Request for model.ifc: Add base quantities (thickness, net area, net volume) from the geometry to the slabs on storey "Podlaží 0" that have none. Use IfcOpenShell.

First a look at what the model holds.

```python
import ifcopenshell
import ifcopenshell.util.element
import ifcopenshell.util.unit

model = ifcopenshell.open("model.ifc")
print(model.schema)
for unit_type in ("LENGTHUNIT", "AREAUNIT", "VOLUMEUNIT"):
    print(unit_type, ifcopenshell.util.unit.calculate_unit_scale(model, unit_type))
storey = next(s for s in model.by_type("IfcBuildingStorey") if s.Name == "Podlaží 0")
slabs = [e for e in ifcopenshell.util.element.get_decomposition(storey) if e.is_a("IfcSlab")]
for e in sorted(slabs, key=lambda e: e.id()):
    print(e.id(), e.is_a(), e.Name, list(ifcopenshell.util.element.get_psets(e, qtos_only=True)), sep=" | ")
```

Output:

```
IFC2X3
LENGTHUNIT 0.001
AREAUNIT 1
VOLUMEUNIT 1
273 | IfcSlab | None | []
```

```python
import ifcopenshell
import ifcopenshell.api.pset
import ifcopenshell.geom
import ifcopenshell.util.element
import ifcopenshell.util.shape
import ifcopenshell.util.unit

model = ifcopenshell.open("model.ifc")
unit_scale = ifcopenshell.util.unit.calculate_unit_scale(model)
area_scale = ifcopenshell.util.unit.calculate_unit_scale(model, "AREAUNIT")
volume_scale = ifcopenshell.util.unit.calculate_unit_scale(model, "VOLUMEUNIT")
settings = ifcopenshell.geom.settings()

storey = next(s for s in model.by_type("IfcBuildingStorey") if s.Name == "Podlaží 0")
slabs = [e for e in ifcopenshell.util.element.get_decomposition(storey) if e.is_a("IfcSlab")]

for e in sorted(slabs, key=lambda e: e.id()):
    if ifcopenshell.util.element.get_psets(e, qtos_only=True, should_inherit=False):
        continue
    # Geometry comes back in metres, in the element's own axes.
    shape = ifcopenshell.geom.create_shape(settings, e)
    values = {
        "Width": ifcopenshell.util.shape.get_z(shape.geometry) / unit_scale,
        "NetArea": ifcopenshell.util.shape.get_footprint_area(shape.geometry) / area_scale,
        "NetVolume": ifcopenshell.util.shape.get_volume(shape.geometry) / volume_scale,
    }
    qto = ifcopenshell.api.pset.add_qto(model, product=e, name="BaseQuantities")
    ifcopenshell.api.pset.edit_qto(model, qto=qto, properties=values)
    print(e.id(), {k: round(v, 3) for k, v in values.items()})

model.write("model-out.ifc")
```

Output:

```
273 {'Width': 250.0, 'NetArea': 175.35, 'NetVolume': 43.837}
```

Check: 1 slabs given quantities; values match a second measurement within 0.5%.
